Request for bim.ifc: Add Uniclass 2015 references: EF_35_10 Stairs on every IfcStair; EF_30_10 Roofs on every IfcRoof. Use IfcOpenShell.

First a look at what the model holds.

```python
import ifcopenshell

model = ifcopenshell.open("bim.ifc")
print(model.schema)
print("classifications:", [c.Name for c in model.by_type("IfcClassification")])
for ifc_class in ("IfcDoor", "IfcRoof", "IfcStair", "IfcWall", "IfcWindow"):
    print(ifc_class, len(model.by_type(ifc_class)))
```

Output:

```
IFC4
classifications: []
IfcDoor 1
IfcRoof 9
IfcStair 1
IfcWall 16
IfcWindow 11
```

```python
import ifcopenshell
import ifcopenshell.api.classification

model = ifcopenshell.open("bim.ifc")

system = ifcopenshell.api.classification.add_classification(model, classification="Uniclass 2015")

codes = {
    "IfcStair": ("EF_35_10", "Stairs"),
    "IfcRoof": ("EF_30_10", "Roofs"),
}
for ifc_class, (code, name) in codes.items():
    products = model.by_type(ifc_class)
    ifcopenshell.api.classification.add_reference(
        model, products=products, classification=system, identification=code, name=name
    )
    print(code, len(products))

model.write("bim_v2.ifc")
```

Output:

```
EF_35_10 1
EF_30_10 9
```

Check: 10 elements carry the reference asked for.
